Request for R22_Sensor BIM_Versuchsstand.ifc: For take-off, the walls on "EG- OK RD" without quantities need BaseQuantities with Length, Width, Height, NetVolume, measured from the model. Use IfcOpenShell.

First a look at what the model holds.

```python
import ifcopenshell
import ifcopenshell.util.element
import ifcopenshell.util.unit

model = ifcopenshell.open("R22_Sensor BIM_Versuchsstand.ifc")
print(model.schema)
for unit_type in ("LENGTHUNIT", "AREAUNIT", "VOLUMEUNIT"):
    print(unit_type, ifcopenshell.util.unit.calculate_unit_scale(model, unit_type))
storey = next(s for s in model.by_type("IfcBuildingStorey") if s.Name == "EG- OK RD")
walls = [e for e in ifcopenshell.util.element.get_decomposition(storey) if e.is_a("IfcWall")]
for e in sorted(walls, key=lambda e: e.id()):
    print(e.id(), e.is_a(), e.Name, list(ifcopenshell.util.element.get_psets(e, qtos_only=True)), sep=" | ")
```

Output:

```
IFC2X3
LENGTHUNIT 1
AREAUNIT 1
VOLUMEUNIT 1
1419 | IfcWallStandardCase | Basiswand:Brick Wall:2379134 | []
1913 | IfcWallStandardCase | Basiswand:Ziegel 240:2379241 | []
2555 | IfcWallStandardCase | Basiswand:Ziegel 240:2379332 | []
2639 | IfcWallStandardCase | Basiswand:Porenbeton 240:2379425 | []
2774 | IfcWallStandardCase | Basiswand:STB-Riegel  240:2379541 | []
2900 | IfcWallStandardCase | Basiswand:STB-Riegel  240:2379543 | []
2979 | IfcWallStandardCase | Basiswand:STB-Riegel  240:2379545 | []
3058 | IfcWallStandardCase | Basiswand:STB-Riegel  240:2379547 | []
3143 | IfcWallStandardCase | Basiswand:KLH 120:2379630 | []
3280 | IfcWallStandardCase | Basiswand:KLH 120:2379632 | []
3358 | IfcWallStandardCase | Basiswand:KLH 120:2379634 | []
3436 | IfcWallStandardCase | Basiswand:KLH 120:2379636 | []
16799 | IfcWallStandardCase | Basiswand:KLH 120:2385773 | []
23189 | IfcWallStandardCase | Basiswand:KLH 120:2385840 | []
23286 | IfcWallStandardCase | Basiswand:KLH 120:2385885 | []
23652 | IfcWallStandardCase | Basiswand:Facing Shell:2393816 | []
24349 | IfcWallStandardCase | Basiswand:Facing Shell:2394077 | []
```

```python
import ifcopenshell
import ifcopenshell.api.pset
import ifcopenshell.geom
import ifcopenshell.util.element
import ifcopenshell.util.shape
import ifcopenshell.util.unit

model = ifcopenshell.open("R22_Sensor BIM_Versuchsstand.ifc")
unit_scale = ifcopenshell.util.unit.calculate_unit_scale(model)
volume_scale = ifcopenshell.util.unit.calculate_unit_scale(model, "VOLUMEUNIT")
settings = ifcopenshell.geom.settings()

storey = next(s for s in model.by_type("IfcBuildingStorey") if s.Name == "EG- OK RD")
walls = [e for e in ifcopenshell.util.element.get_decomposition(storey) if e.is_a("IfcWall")]

for e in sorted(walls, key=lambda e: e.id()):
    if ifcopenshell.util.element.get_psets(e, qtos_only=True, should_inherit=False):
        continue
    # Geometry comes back in metres, in the element's own axes.
    shape = ifcopenshell.geom.create_shape(settings, e)
    values = {
        "Length": ifcopenshell.util.shape.get_x(shape.geometry) / unit_scale,
        "Width": ifcopenshell.util.shape.get_y(shape.geometry) / unit_scale,
        "Height": ifcopenshell.util.shape.get_z(shape.geometry) / unit_scale,
        "NetVolume": ifcopenshell.util.shape.get_volume(shape.geometry) / volume_scale,
    }
    qto = ifcopenshell.api.pset.add_qto(model, product=e, name="BaseQuantities")
    ifcopenshell.api.pset.edit_qto(model, qto=qto, properties=values)
    print(e.id(), {k: round(v, 3) for k, v in values.items()})

model.write("R22_Sensor BIM_Versuchsstand_edited.ifc")
```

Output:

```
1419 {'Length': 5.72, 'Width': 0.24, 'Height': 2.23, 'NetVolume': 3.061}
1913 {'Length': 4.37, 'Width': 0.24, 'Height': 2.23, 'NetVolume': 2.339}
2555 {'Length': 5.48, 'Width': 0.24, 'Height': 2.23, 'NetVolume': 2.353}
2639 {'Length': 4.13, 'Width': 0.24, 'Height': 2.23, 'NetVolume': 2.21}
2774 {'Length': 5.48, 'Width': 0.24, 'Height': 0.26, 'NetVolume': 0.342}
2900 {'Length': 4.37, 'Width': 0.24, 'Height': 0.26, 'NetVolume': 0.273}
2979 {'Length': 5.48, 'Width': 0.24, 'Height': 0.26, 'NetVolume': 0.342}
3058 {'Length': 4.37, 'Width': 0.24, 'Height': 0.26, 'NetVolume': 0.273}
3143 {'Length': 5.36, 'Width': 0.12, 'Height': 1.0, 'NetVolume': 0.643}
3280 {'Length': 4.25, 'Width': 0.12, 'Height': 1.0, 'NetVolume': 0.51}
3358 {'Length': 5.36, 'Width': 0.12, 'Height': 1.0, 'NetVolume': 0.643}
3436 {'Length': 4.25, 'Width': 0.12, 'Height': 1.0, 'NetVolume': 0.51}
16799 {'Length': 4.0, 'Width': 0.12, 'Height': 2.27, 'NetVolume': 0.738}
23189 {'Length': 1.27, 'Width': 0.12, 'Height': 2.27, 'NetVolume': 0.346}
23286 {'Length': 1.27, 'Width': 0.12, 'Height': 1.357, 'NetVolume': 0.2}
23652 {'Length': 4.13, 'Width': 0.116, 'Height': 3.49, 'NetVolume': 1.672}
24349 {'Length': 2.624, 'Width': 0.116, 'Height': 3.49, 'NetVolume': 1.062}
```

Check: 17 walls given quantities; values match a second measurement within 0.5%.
